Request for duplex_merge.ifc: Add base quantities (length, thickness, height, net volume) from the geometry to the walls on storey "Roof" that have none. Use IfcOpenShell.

First a look at what the model holds.

```python
import ifcopenshell
import ifcopenshell.util.element
import ifcopenshell.util.unit

model = ifcopenshell.open("duplex_merge.ifc")
print(model.schema)
for unit_type in ("LENGTHUNIT", "AREAUNIT", "VOLUMEUNIT"):
    print(unit_type, ifcopenshell.util.unit.calculate_unit_scale(model, unit_type))
storey = next(s for s in model.by_type("IfcBuildingStorey") if s.Name == "Roof")
walls = [e for e in ifcopenshell.util.element.get_decomposition(storey) if e.is_a("IfcWall")]
for e in sorted(walls, key=lambda e: e.id()):
    print(e.id(), e.is_a(), e.Name, list(ifcopenshell.util.element.get_psets(e, qtos_only=True)), sep=" | ")
```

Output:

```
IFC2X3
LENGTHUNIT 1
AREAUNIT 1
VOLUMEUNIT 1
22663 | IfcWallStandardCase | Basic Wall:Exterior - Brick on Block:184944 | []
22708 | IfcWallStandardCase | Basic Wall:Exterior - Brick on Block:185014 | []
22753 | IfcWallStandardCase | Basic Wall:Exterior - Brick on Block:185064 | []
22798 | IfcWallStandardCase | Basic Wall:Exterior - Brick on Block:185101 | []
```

```python
import ifcopenshell
import ifcopenshell.api.pset
import ifcopenshell.geom
import ifcopenshell.util.element
import ifcopenshell.util.shape
import ifcopenshell.util.unit

model = ifcopenshell.open("duplex_merge.ifc")
unit_scale = ifcopenshell.util.unit.calculate_unit_scale(model)
volume_scale = ifcopenshell.util.unit.calculate_unit_scale(model, "VOLUMEUNIT")
settings = ifcopenshell.geom.settings()

storey = next(s for s in model.by_type("IfcBuildingStorey") if s.Name == "Roof")
walls = [e for e in ifcopenshell.util.element.get_decomposition(storey) if e.is_a("IfcWall")]

for e in sorted(walls, key=lambda e: e.id()):
    if ifcopenshell.util.element.get_psets(e, qtos_only=True, should_inherit=False):
        continue
    # Geometry comes back in metres, in the element's own axes.
    shape = ifcopenshell.geom.create_shape(settings, e)
    values = {
        "Length": ifcopenshell.util.shape.get_x(shape.geometry) / unit_scale,
        "Width": ifcopenshell.util.shape.get_y(shape.geometry) / unit_scale,
        "Height": ifcopenshell.util.shape.get_z(shape.geometry) / unit_scale,
        "NetVolume": ifcopenshell.util.shape.get_volume(shape.geometry) / volume_scale,
    }
    qto = ifcopenshell.api.pset.add_qto(model, product=e, name="BaseQuantities")
    ifcopenshell.api.pset.edit_qto(model, qto=qto, properties=values)
    print(e.id(), {k: round(v, 3) for k, v in values.items()})

model.write("duplex_merge-out.ifc")
```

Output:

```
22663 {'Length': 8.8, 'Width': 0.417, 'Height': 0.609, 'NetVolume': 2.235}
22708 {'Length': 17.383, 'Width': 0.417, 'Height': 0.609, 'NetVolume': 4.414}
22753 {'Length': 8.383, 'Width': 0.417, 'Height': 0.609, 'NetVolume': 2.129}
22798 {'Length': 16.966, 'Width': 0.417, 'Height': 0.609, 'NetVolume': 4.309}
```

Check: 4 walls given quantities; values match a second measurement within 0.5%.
